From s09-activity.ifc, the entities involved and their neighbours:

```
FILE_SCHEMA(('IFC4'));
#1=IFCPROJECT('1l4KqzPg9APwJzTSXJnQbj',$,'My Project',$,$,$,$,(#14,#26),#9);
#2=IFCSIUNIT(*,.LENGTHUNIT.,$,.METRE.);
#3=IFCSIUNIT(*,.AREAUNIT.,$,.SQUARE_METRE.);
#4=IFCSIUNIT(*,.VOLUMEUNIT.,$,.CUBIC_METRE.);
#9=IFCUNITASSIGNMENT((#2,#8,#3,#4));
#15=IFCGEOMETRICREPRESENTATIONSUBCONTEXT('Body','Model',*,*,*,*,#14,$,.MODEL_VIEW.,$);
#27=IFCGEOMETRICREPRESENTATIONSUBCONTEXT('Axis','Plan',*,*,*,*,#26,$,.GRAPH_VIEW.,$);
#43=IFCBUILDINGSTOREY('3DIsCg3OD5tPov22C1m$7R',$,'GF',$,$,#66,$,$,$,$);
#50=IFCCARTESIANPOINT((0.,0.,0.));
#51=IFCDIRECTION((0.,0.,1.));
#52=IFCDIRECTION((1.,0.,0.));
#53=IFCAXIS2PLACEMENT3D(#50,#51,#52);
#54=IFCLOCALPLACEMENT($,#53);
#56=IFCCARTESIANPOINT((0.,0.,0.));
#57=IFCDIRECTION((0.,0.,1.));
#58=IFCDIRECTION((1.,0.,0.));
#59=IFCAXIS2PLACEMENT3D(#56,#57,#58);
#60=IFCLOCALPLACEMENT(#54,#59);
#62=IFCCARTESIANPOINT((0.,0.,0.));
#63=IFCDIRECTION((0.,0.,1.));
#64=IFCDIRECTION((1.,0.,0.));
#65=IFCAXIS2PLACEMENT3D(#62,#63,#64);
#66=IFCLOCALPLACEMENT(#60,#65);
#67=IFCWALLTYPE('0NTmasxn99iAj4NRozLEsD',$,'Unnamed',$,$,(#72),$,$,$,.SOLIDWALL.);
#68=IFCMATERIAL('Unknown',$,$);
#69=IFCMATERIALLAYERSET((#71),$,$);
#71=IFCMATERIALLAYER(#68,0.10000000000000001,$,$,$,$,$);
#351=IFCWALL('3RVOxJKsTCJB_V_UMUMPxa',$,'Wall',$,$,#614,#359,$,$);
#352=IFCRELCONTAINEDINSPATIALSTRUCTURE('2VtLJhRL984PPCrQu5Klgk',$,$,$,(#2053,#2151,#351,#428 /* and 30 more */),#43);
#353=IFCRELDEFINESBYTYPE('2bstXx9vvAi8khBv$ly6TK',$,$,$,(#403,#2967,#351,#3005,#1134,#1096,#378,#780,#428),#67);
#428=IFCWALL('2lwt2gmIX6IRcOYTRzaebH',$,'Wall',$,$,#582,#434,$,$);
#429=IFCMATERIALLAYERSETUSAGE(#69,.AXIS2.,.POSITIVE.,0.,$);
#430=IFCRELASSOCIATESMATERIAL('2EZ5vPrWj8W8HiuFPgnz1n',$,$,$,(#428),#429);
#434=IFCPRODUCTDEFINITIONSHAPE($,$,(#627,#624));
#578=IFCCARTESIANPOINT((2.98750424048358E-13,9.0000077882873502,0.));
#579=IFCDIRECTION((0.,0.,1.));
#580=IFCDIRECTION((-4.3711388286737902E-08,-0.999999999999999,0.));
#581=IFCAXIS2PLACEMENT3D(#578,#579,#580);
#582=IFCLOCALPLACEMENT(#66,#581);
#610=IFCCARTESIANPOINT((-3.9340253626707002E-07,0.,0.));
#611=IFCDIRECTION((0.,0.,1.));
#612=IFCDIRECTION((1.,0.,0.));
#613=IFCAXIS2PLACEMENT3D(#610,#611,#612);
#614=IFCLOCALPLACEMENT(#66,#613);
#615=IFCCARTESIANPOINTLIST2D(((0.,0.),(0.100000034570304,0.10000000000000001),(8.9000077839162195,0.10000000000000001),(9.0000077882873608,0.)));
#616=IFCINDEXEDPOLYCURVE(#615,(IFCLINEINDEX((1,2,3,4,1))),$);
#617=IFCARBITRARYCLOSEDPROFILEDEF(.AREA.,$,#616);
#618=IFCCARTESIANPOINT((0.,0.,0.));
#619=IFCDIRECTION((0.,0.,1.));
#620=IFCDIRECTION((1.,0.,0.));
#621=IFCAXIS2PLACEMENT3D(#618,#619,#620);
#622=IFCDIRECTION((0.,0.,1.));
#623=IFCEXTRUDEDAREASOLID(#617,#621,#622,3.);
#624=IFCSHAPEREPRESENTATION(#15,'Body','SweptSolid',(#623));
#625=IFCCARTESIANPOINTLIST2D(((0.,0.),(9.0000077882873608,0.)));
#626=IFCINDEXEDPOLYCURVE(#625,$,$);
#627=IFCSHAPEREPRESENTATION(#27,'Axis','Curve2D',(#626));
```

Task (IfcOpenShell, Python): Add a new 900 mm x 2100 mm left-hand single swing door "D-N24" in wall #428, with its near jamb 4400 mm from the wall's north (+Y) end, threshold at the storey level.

```python
import numpy as np
import ifcopenshell
import ifcopenshell.api.feature
import ifcopenshell.api.geometry
import ifcopenshell.api.root
import ifcopenshell.api.spatial
import ifcopenshell.geom
import ifcopenshell.util.element
import ifcopenshell.util.placement
import ifcopenshell.util.representation
import ifcopenshell.util.shape
import ifcopenshell.util.unit

model = ifcopenshell.open("s09-activity.ifc")
unit_scale = ifcopenshell.util.unit.calculate_unit_scale(model)
settings = ifcopenshell.geom.settings()


def volume(element):
    """Net volume in cubic metres, openings subtracted."""
    shape = ifcopenshell.geom.create_shape(settings, element)
    return ifcopenshell.util.shape.get_volume(shape.geometry)


wall = model.by_guid("2lwt2gmIX6IRcOYTRzaebH")
storey = ifcopenshell.util.element.get_container(wall, ifc_class="IfcBuildingStorey")
context = ifcopenshell.util.representation.get_context(model, "Model", "Body", "MODEL_VIEW")
before = volume(wall)

width, height, from_end, sill = 0.9, 2.1, 4.4, 0.0  # metres

# The wall runs along its own X axis, and the end named is its -X end.
wall_shape = ifcopenshell.geom.create_shape(settings, wall)
x, y, z = ifcopenshell.util.shape.get_vertices(wall_shape.geometry).T
start = x.min() + from_end
face, thickness = float(y.min()), float(y.max() - y.min())
wall_matrix = ifcopenshell.util.placement.get_local_placement(wall.ObjectPlacement)
level = ifcopenshell.util.placement.get_local_placement(storey.ObjectPlacement)[2, 3]


def in_wall(x, y):
    """Placement at x, y metres in the wall's axes, at sill height."""
    matrix = wall_matrix.copy()
    matrix[:, 3] = wall_matrix @ np.array([x / unit_scale, y / unit_scale, 0.0, 1.0])
    matrix[2, 3] = level + sill / unit_scale
    return matrix


# Opening: a box that overshoots both wall faces by 50 mm.
opening = ifcopenshell.api.root.create_entity(model, ifc_class="IfcOpeningElement", predefined_type="OPENING")
box = ifcopenshell.api.geometry.add_wall_representation(
    model, context=context, length=width, height=height, thickness=thickness + 0.1
)
ifcopenshell.api.geometry.assign_representation(model, product=opening, representation=box)
ifcopenshell.api.geometry.edit_object_placement(model, product=opening, matrix=in_wall(start, face - 0.05), is_si=False)
ifcopenshell.api.feature.add_feature(model, feature=opening, element=wall)

door = ifcopenshell.api.root.create_entity(model, ifc_class="IfcDoor", name="D-N24", predefined_type="DOOR")
door.OverallWidth, door.OverallHeight = width / unit_scale, height / unit_scale
door.OperationType = "SINGLE_SWING_LEFT"
body = ifcopenshell.api.geometry.add_door_representation(
    model,
    context=context,
    overall_width=door.OverallWidth,
    overall_height=door.OverallHeight,
    operation_type="SINGLE_SWING_LEFT",
    lining_properties={"LiningDepth": thickness / unit_scale, "ThresholdDepth": thickness / unit_scale},
)
ifcopenshell.api.geometry.assign_representation(model, product=door, representation=body)
ifcopenshell.api.spatial.assign_container(model, products=[door], relating_structure=storey)
ifcopenshell.api.feature.add_filling(model, opening=opening, element=door)

# The lining spans the wall, so the door starts at the wall face.
ifcopenshell.api.geometry.edit_object_placement(model, product=door, matrix=in_wall(start, face), is_si=False)

after = volume(wall)

print(f"wall volume {before:.3f} -> {after:.3f} m3")

model.write("s09-activity_edited.ifc")
```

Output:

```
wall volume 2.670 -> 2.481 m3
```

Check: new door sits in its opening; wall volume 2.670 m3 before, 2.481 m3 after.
